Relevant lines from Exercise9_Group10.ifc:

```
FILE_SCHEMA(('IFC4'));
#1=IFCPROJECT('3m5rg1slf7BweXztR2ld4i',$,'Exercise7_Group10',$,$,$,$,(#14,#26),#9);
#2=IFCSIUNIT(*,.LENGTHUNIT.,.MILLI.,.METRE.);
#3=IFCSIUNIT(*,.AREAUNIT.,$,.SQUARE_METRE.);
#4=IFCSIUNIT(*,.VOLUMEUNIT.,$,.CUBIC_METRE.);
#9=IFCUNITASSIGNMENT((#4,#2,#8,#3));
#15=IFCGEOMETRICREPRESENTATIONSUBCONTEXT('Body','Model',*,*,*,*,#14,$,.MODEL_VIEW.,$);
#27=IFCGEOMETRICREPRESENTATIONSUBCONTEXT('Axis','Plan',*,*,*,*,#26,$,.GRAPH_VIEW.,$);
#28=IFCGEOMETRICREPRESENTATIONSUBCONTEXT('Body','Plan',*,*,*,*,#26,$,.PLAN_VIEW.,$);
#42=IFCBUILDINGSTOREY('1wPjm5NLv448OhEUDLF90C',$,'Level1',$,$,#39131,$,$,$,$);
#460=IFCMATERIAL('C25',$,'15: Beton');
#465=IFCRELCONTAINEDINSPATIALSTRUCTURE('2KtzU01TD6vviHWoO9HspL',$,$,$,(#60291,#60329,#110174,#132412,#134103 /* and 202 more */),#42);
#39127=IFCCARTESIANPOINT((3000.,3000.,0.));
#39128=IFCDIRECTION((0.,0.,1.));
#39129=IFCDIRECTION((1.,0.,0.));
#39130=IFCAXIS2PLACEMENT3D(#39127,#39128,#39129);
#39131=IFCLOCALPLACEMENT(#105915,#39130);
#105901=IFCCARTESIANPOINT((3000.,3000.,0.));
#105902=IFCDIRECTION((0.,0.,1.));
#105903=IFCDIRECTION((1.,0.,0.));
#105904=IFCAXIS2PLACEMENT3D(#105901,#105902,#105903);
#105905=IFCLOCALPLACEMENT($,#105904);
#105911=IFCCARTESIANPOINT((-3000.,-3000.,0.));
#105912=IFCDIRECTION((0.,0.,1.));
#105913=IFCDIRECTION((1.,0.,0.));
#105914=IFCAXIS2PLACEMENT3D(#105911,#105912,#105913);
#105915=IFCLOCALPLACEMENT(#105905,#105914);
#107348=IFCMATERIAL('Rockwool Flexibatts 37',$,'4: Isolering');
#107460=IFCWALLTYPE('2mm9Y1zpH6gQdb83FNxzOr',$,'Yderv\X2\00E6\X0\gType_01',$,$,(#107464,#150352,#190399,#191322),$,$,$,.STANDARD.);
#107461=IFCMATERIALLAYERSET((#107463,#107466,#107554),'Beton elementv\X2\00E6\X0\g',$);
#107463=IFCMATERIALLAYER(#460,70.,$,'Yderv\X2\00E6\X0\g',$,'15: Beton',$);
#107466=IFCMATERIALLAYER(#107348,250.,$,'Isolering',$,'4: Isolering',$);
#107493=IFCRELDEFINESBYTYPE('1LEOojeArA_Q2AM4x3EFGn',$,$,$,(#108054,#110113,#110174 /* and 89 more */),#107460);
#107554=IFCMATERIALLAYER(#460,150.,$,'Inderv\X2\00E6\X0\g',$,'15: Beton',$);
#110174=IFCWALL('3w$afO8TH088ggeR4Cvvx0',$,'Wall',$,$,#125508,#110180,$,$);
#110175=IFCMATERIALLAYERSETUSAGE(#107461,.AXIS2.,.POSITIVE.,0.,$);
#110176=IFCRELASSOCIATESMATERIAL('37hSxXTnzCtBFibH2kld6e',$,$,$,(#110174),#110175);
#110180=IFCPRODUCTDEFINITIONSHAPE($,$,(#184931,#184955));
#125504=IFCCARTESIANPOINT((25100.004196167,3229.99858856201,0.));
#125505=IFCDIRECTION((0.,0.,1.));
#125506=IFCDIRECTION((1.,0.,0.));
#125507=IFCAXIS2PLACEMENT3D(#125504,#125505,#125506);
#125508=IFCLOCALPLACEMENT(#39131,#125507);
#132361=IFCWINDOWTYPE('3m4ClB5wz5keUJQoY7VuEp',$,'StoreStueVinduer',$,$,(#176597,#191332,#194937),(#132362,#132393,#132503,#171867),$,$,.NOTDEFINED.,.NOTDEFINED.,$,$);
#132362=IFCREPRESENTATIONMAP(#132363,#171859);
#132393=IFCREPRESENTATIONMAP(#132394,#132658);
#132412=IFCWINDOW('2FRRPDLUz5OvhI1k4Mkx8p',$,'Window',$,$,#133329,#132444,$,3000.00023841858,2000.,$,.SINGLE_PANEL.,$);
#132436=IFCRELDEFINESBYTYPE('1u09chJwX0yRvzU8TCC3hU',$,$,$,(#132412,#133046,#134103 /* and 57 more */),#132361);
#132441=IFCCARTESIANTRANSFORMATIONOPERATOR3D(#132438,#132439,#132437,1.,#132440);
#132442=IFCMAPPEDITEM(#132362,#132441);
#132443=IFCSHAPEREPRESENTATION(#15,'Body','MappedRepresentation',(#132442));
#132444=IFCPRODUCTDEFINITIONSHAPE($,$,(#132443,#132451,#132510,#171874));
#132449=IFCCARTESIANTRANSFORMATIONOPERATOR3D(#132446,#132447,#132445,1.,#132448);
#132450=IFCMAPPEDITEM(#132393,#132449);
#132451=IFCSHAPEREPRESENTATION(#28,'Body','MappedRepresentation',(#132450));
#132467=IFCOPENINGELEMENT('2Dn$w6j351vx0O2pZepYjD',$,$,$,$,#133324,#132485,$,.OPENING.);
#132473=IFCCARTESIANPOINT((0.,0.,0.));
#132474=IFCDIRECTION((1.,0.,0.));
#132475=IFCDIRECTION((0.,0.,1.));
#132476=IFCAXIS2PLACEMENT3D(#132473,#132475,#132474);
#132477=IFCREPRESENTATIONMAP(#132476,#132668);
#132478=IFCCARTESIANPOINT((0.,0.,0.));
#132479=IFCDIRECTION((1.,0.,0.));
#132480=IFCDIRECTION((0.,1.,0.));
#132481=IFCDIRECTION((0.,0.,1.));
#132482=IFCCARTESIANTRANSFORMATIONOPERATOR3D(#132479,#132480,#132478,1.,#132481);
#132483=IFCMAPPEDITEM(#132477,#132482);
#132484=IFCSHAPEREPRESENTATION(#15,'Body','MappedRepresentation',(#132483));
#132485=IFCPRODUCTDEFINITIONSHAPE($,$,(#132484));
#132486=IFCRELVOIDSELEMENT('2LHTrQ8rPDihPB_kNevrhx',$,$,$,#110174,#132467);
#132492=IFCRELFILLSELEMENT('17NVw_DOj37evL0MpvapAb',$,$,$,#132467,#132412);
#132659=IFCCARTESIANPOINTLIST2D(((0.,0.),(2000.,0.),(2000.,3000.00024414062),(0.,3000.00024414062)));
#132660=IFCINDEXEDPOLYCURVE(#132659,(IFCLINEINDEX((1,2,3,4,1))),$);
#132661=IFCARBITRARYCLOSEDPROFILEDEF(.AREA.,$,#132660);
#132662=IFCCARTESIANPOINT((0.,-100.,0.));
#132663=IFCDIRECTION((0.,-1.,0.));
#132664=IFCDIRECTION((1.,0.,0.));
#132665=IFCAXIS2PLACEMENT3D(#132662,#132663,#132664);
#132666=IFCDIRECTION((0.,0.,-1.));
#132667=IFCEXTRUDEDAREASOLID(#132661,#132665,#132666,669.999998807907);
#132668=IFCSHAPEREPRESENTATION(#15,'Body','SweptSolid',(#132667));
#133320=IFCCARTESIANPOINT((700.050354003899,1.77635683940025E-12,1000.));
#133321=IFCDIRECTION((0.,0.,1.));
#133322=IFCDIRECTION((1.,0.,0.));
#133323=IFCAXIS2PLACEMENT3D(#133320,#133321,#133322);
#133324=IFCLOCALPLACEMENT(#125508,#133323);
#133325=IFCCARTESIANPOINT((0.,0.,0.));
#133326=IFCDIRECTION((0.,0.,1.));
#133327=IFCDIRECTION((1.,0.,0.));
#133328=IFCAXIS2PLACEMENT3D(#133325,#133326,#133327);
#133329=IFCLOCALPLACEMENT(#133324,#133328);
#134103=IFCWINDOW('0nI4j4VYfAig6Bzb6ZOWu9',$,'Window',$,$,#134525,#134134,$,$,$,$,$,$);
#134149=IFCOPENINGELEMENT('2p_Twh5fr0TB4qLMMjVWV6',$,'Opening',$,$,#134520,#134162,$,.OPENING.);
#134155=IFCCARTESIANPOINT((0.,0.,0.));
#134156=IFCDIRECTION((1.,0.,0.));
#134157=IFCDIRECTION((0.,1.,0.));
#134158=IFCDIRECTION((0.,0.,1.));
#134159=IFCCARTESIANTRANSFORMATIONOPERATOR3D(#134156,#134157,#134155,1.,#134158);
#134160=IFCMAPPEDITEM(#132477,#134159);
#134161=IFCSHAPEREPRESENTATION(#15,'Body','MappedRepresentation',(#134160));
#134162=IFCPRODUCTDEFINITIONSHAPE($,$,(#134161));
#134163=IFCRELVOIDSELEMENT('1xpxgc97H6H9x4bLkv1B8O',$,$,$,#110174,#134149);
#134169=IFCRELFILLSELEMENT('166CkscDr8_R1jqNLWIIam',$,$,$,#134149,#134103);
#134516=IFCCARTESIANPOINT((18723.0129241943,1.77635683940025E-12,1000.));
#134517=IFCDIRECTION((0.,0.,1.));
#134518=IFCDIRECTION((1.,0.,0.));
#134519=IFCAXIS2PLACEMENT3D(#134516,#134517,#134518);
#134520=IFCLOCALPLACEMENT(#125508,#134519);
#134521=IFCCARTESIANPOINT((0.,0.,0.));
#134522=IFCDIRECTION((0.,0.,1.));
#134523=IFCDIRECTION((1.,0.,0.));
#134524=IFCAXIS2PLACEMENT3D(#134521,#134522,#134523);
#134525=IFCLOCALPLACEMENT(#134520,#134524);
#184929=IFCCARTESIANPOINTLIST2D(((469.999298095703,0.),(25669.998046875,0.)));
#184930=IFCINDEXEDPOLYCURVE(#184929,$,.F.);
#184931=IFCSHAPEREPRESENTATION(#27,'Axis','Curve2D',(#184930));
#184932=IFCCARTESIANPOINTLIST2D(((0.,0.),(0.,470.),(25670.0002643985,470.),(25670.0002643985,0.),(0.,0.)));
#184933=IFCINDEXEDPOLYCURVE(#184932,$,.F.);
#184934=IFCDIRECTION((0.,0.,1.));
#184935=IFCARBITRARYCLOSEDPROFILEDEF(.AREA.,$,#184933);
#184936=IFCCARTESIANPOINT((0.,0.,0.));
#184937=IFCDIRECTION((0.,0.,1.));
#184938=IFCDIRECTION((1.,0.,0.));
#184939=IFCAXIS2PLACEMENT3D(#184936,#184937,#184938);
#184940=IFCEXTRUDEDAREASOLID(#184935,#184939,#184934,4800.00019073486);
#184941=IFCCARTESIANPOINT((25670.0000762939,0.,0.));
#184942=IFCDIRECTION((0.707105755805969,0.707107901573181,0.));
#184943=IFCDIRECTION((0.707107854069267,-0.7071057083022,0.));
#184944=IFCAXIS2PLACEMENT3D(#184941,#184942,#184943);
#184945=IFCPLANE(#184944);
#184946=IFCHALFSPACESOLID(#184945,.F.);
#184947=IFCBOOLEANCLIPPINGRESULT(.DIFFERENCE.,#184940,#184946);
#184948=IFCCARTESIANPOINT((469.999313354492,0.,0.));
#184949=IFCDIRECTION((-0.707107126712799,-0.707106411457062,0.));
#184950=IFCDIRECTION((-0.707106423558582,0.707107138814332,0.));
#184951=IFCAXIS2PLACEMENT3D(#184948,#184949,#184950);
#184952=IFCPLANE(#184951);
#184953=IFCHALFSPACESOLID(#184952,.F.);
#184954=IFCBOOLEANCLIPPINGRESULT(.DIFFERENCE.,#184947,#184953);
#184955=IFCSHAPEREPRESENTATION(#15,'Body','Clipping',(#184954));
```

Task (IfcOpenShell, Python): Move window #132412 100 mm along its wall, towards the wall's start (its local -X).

```python
import ifcopenshell
import ifcopenshell.api.geometry
import ifcopenshell.util.placement
import ifcopenshell.util.unit

model = ifcopenshell.open("Exercise9_Group10.ifc")
unit_scale = ifcopenshell.util.unit.calculate_unit_scale(model)

window = model.by_guid("2FRRPDLUz5OvhI1k4Mkx8p")
opening = window.FillsVoids[0].RelatingOpeningElement
wall = opening.VoidsElements[0].RelatingBuildingElement

wall_matrix = ifcopenshell.util.placement.get_local_placement(wall.ObjectPlacement)
shift = wall_matrix[:3, 0] * -0.1 / unit_scale
before = ifcopenshell.util.placement.get_local_placement(window.ObjectPlacement)[:3, 3].copy()

# The window is placed relative to its opening, so it follows when the opening moves.
matrix = ifcopenshell.util.placement.get_local_placement(opening.ObjectPlacement)
matrix[:3, 3] += shift
ifcopenshell.api.geometry.edit_object_placement(
    model, product=opening, matrix=matrix, is_si=False, should_transform_children=True
)

after = ifcopenshell.util.placement.get_local_placement(window.ObjectPlacement)[:3, 3]
print("window moved by", (after - before).round(3) + 0.0)

model.write("Exercise9_Group10_v2.ifc")
```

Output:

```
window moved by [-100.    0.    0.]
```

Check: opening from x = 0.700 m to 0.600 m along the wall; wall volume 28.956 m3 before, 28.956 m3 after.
